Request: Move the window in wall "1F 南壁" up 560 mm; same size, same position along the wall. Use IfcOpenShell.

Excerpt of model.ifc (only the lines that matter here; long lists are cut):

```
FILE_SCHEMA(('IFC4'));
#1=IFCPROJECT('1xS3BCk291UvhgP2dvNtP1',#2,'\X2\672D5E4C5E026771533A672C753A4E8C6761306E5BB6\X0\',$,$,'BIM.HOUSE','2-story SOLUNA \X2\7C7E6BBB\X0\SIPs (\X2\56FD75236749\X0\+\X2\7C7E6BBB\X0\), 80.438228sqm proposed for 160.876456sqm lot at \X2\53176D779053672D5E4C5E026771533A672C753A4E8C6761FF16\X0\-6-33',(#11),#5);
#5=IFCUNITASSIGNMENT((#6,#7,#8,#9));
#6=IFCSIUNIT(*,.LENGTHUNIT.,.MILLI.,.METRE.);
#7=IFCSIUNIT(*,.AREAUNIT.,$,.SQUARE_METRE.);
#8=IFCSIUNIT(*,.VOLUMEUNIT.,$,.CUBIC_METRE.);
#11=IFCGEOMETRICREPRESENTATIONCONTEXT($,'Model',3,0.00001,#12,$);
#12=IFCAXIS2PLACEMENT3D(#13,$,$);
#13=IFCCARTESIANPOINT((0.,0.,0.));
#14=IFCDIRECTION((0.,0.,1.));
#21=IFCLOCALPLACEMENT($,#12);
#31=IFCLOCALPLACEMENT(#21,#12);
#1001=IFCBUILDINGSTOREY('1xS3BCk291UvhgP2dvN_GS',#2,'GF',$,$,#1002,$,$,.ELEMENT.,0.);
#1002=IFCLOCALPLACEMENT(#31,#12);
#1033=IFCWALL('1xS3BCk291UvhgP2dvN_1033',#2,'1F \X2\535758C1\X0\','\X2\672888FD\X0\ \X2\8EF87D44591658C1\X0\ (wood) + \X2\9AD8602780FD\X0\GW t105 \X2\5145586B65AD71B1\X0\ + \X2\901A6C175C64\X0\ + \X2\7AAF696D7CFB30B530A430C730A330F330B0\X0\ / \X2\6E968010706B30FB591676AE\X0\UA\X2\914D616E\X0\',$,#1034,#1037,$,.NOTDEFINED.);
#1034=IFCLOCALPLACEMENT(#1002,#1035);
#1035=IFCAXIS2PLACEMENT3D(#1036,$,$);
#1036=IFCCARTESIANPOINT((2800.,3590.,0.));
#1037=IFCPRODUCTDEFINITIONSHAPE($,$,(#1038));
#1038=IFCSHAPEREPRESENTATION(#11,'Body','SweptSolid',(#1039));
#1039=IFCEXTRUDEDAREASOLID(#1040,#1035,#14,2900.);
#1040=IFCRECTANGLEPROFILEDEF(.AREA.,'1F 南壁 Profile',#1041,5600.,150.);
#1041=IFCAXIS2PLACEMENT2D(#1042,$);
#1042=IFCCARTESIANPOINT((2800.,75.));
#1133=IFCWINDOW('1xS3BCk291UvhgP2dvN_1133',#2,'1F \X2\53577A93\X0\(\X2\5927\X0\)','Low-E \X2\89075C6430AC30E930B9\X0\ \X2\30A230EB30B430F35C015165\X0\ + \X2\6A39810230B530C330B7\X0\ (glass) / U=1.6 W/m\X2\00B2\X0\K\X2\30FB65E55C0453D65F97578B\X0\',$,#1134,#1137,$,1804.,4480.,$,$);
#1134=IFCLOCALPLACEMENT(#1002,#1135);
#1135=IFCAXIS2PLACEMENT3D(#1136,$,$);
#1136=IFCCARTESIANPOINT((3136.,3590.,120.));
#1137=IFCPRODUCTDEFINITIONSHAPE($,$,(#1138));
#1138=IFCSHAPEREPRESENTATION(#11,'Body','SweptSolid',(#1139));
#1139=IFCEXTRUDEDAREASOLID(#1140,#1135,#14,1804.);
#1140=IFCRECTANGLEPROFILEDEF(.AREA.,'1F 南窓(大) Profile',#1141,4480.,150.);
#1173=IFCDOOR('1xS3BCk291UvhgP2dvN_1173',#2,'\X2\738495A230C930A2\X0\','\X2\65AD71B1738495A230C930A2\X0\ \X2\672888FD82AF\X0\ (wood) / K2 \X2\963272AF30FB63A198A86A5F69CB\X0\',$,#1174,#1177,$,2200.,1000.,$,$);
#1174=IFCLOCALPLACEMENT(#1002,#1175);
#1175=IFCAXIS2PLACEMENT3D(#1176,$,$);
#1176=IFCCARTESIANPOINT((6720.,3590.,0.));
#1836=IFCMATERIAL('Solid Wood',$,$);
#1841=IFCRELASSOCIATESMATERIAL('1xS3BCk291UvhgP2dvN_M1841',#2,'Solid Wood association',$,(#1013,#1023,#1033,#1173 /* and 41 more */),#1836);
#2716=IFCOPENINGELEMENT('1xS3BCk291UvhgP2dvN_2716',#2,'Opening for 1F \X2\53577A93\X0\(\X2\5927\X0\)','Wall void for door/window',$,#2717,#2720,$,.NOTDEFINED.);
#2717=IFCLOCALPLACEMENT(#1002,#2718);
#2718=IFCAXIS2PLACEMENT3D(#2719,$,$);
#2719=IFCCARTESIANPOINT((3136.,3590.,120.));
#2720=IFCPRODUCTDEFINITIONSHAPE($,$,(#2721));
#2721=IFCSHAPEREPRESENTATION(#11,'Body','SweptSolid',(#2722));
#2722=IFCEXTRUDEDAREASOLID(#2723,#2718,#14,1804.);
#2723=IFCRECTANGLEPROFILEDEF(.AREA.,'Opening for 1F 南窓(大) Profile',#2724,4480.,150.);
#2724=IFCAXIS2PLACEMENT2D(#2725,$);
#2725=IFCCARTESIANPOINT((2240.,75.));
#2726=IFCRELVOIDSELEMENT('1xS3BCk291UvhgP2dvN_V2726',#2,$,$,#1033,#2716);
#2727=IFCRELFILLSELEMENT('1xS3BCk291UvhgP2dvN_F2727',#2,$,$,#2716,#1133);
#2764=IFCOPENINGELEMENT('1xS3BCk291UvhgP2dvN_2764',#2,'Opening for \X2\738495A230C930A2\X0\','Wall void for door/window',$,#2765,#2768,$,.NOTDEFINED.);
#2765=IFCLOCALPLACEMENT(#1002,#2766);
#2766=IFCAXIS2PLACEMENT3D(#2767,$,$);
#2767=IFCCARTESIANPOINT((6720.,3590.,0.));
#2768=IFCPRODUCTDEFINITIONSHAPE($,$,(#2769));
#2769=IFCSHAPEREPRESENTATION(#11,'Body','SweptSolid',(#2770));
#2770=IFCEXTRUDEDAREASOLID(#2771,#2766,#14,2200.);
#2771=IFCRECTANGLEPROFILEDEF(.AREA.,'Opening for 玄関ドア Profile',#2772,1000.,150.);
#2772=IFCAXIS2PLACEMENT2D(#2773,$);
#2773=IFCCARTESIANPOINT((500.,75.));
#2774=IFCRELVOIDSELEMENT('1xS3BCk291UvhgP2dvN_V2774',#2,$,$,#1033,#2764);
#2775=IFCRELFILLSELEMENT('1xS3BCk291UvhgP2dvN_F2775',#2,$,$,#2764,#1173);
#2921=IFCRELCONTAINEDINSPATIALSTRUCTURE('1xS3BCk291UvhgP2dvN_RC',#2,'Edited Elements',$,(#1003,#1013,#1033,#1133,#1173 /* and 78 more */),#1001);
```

```python
import numpy as np
import ifcopenshell
import ifcopenshell.api.geometry
import ifcopenshell.util.placement
import ifcopenshell.util.unit

model = ifcopenshell.open("model.ifc")
unit_scale = ifcopenshell.util.unit.calculate_unit_scale(model)

window = model.by_guid("1xS3BCk291UvhgP2dvN_1133")
opening = window.FillsVoids[0].RelatingOpeningElement
dz = 560.0

shift = np.array([0.0, 0.0, dz])
# The window is not placed relative to its opening, so move both.
for product in (opening, window):
    matrix = ifcopenshell.util.placement.get_local_placement(product.ObjectPlacement)
    matrix[:3, 3] += shift
    ifcopenshell.api.geometry.edit_object_placement(model, product=product, matrix=matrix, is_si=False)

print(f"moved by {dz * unit_scale:+.3f} m")

model.write("model_rev.ifc")
```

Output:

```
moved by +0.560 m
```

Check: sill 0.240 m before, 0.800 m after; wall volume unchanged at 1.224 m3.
